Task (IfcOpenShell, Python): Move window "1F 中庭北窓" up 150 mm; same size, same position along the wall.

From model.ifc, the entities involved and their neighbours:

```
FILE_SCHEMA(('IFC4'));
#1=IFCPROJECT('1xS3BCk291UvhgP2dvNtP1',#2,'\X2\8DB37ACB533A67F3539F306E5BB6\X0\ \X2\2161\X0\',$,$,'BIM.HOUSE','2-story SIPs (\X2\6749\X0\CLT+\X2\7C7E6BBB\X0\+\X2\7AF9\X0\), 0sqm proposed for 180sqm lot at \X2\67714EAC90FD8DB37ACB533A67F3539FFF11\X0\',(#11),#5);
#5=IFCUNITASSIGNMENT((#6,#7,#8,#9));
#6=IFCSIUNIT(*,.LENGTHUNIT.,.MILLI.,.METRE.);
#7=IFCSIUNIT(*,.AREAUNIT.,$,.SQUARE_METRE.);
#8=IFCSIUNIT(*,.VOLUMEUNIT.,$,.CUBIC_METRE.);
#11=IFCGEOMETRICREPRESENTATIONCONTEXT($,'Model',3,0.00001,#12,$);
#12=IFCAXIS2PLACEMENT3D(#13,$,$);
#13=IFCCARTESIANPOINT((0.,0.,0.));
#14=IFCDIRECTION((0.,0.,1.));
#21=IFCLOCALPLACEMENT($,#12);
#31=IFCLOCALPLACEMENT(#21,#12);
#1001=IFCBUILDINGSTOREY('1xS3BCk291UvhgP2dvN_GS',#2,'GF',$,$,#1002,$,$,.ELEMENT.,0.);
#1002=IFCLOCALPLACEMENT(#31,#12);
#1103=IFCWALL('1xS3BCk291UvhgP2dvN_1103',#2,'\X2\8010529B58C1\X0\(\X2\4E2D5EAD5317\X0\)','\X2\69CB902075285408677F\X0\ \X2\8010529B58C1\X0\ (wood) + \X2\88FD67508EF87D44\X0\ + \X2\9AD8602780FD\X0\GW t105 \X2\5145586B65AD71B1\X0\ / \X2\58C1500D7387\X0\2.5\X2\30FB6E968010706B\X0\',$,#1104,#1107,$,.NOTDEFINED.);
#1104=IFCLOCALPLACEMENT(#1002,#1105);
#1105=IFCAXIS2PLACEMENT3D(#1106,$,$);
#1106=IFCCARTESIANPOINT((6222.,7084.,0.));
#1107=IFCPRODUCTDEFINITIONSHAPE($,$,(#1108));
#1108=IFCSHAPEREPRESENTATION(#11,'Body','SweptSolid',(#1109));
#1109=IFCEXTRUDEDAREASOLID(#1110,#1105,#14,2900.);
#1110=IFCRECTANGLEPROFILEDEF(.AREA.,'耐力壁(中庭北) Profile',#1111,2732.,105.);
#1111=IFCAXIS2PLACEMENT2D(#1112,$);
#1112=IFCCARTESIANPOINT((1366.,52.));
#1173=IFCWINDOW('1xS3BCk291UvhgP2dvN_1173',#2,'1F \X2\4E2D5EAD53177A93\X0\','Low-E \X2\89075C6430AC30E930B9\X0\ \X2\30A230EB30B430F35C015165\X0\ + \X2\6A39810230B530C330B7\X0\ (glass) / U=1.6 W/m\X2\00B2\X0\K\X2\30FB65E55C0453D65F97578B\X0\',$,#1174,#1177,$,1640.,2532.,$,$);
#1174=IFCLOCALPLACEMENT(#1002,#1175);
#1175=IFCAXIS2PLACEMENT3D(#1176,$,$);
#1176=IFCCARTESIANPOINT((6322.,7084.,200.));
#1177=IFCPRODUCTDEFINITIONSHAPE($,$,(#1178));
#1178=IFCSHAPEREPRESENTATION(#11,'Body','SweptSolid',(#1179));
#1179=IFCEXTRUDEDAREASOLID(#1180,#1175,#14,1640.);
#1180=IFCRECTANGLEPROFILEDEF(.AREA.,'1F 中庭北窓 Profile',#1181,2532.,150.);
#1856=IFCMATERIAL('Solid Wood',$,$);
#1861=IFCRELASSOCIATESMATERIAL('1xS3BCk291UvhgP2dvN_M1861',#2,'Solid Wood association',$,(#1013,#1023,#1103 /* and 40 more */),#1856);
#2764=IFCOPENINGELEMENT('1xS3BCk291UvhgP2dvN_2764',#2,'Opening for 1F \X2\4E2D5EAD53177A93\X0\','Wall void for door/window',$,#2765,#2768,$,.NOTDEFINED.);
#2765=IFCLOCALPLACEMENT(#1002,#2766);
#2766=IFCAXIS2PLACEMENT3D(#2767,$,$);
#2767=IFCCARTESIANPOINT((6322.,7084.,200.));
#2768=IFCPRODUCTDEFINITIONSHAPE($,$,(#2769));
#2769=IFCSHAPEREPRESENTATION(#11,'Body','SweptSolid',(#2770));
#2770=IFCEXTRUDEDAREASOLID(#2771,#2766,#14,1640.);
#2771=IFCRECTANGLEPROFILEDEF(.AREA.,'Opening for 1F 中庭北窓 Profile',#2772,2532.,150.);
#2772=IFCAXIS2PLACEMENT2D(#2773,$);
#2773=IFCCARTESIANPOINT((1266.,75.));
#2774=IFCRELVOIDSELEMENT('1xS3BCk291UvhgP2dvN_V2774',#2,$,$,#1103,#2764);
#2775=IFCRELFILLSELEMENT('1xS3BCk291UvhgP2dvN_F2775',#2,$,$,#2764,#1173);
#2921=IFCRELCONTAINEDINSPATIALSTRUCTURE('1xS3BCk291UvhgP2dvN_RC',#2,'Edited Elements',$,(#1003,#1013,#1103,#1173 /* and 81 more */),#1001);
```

```python
import numpy as np
import ifcopenshell
import ifcopenshell.api.geometry
import ifcopenshell.util.placement
import ifcopenshell.util.unit

model = ifcopenshell.open("model.ifc")
unit_scale = ifcopenshell.util.unit.calculate_unit_scale(model)

window = model.by_guid("1xS3BCk291UvhgP2dvN_1173")
opening = window.FillsVoids[0].RelatingOpeningElement
dz = 150.0

shift = np.array([0.0, 0.0, dz])
# The window is not placed relative to its opening, so move both.
for product in (opening, window):
    matrix = ifcopenshell.util.placement.get_local_placement(product.ObjectPlacement)
    matrix[:3, 3] += shift
    ifcopenshell.api.geometry.edit_object_placement(model, product=product, matrix=matrix, is_si=False)

print(f"moved by {dz * unit_scale:+.3f} m")

model.write("model_rev.ifc")
```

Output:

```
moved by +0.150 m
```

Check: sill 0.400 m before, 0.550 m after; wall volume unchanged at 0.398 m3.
